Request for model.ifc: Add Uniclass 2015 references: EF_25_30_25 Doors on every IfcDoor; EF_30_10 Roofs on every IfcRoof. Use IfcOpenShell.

First a look at what the model holds.

```python
import ifcopenshell

model = ifcopenshell.open("model.ifc")
print(model.schema)
print("classifications:", [c.Name for c in model.by_type("IfcClassification")])
for ifc_class in ("IfcDoor", "IfcRoof", "IfcStair", "IfcWall", "IfcWindow"):
    print(ifc_class, len(model.by_type(ifc_class)))
```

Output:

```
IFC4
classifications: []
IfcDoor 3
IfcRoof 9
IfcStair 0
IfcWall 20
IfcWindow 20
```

```python
import ifcopenshell
import ifcopenshell.api.classification

model = ifcopenshell.open("model.ifc")

system = ifcopenshell.api.classification.add_classification(model, classification="Uniclass 2015")

codes = {
    "IfcDoor": ("EF_25_30_25", "Doors"),
    "IfcRoof": ("EF_30_10", "Roofs"),
}
for ifc_class, (code, name) in codes.items():
    products = model.by_type(ifc_class)
    ifcopenshell.api.classification.add_reference(
        model, products=products, classification=system, identification=code, name=name
    )
    print(code, len(products))

model.write("model-out.ifc")
```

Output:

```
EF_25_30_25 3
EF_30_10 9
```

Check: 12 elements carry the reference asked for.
